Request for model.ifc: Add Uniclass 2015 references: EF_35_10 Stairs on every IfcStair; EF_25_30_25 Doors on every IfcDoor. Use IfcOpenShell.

First a look at what the model holds.

```python
import ifcopenshell

model = ifcopenshell.open("model.ifc")
print(model.schema)
print("classifications:", [c.Name for c in model.by_type("IfcClassification")])
for ifc_class in ("IfcDoor", "IfcRoof", "IfcStair", "IfcWall", "IfcWindow"):
    print(ifc_class, len(model.by_type(ifc_class)))
```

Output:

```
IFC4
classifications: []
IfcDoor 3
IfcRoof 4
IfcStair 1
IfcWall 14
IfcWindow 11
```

```python
import ifcopenshell
import ifcopenshell.api.classification

model = ifcopenshell.open("model.ifc")

system = ifcopenshell.api.classification.add_classification(model, classification="Uniclass 2015")

codes = {
    "IfcStair": ("EF_35_10", "Stairs"),
    "IfcDoor": ("EF_25_30_25", "Doors"),
}
for ifc_class, (code, name) in codes.items():
    products = model.by_type(ifc_class)
    ifcopenshell.api.classification.add_reference(
        model, products=products, classification=system, identification=code, name=name
    )
    print(code, len(products))

model.write("model_rev.ifc")
```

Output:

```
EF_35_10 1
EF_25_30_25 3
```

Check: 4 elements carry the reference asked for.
